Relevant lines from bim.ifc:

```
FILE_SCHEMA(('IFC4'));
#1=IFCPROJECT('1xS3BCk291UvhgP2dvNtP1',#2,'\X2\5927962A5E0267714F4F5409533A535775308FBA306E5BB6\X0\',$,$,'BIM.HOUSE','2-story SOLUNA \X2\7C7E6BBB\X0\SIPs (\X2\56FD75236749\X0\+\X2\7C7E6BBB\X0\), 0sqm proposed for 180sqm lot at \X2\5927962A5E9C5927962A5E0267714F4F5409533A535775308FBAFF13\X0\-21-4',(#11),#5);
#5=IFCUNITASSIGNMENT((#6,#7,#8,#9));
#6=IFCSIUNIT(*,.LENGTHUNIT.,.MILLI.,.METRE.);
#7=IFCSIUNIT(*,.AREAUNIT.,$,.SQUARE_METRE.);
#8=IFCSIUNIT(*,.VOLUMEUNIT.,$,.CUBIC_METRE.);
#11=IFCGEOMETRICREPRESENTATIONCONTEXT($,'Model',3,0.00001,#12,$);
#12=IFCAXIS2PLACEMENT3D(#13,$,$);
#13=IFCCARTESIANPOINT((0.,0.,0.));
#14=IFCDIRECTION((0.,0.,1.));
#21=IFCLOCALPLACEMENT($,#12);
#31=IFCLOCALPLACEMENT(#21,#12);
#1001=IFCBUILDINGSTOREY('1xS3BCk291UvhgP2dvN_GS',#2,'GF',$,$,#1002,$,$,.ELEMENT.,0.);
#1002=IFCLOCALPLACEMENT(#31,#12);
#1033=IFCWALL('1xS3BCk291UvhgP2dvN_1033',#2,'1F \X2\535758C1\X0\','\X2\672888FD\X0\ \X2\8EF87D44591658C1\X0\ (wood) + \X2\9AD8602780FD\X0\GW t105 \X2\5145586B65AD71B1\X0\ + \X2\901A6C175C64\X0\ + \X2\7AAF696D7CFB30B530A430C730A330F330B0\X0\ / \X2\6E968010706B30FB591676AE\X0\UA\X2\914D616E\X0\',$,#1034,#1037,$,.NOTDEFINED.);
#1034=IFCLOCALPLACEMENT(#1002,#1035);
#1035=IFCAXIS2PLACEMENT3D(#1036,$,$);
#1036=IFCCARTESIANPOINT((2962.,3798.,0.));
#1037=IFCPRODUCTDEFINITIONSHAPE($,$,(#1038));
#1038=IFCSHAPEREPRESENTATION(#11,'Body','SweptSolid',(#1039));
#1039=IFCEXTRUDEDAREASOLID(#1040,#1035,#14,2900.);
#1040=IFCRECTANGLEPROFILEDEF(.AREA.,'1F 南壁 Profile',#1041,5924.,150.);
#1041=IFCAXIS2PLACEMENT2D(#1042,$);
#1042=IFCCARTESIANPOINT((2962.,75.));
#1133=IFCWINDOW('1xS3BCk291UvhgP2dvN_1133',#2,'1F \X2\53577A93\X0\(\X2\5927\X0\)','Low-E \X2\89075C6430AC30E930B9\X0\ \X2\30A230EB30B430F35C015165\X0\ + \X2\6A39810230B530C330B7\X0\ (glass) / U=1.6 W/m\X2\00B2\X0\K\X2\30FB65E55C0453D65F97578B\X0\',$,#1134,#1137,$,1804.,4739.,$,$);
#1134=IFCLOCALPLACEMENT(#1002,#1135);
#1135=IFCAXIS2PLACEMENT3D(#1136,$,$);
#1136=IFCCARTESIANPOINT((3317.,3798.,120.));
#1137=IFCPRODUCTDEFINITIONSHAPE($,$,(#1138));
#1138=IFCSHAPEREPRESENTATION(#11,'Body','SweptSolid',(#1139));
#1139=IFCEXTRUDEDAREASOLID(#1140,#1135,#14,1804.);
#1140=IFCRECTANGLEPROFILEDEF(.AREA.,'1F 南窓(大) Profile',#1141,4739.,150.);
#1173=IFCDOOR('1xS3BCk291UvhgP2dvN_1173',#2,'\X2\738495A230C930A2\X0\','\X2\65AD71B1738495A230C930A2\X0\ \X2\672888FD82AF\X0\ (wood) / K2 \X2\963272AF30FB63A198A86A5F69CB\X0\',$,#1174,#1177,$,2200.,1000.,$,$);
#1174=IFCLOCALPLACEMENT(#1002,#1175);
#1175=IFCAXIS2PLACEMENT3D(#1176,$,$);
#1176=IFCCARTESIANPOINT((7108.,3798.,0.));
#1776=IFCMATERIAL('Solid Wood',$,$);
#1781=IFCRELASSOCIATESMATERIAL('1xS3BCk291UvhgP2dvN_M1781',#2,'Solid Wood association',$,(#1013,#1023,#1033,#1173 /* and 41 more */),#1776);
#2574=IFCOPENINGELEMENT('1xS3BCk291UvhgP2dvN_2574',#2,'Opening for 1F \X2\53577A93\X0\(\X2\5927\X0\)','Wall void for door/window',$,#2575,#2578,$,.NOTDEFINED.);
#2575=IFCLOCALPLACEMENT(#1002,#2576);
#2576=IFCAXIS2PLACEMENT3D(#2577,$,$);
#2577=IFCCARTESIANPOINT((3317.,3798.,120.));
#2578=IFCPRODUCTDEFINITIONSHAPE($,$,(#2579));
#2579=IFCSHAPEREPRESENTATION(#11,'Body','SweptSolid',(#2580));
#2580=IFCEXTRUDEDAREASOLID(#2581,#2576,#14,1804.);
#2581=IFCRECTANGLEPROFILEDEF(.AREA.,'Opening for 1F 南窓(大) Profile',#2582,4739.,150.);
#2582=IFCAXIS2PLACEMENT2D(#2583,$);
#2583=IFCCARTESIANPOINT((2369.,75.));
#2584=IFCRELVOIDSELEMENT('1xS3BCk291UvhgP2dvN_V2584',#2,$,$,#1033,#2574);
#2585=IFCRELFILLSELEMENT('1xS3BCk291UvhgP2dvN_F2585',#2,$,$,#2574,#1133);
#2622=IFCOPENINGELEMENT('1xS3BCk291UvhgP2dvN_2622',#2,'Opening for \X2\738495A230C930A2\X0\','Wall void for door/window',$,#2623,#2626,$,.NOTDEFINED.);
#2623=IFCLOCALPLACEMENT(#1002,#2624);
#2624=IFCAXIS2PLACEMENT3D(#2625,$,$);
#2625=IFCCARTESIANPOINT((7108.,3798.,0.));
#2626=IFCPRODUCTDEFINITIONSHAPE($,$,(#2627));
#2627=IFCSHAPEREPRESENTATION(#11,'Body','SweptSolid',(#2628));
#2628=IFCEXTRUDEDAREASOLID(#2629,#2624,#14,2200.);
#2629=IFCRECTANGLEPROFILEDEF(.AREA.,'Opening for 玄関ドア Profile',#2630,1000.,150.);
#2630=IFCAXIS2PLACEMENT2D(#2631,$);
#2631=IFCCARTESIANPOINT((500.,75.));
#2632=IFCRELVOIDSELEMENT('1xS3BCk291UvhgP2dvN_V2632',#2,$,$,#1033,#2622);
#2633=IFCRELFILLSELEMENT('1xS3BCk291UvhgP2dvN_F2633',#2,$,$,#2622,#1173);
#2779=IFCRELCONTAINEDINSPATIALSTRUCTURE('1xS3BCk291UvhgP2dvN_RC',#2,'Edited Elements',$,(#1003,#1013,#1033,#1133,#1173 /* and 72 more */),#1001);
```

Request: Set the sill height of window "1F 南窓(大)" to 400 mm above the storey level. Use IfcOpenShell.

```python
import numpy as np
import ifcopenshell
import ifcopenshell.api.geometry
import ifcopenshell.geom
import ifcopenshell.util.element
import ifcopenshell.util.placement
import ifcopenshell.util.shape
import ifcopenshell.util.unit

model = ifcopenshell.open("bim.ifc")
unit_scale = ifcopenshell.util.unit.calculate_unit_scale(model)

window = model.by_guid("1xS3BCk291UvhgP2dvN_1133")
opening = window.FillsVoids[0].RelatingOpeningElement
storey = ifcopenshell.util.element.get_container(window, ifc_class="IfcBuildingStorey")
level = ifcopenshell.util.placement.get_local_placement(storey.ObjectPlacement)[2, 3]

# The opening's origin need not be at the sill, so measure its lowest point.
shape = ifcopenshell.geom.create_shape(ifcopenshell.geom.settings(), opening)
bottom = ifcopenshell.util.shape.get_shape_bottom_elevation(shape, shape.geometry) / unit_scale
dz = level + 400.0 - bottom

shift = np.array([0.0, 0.0, dz])
# The window is not placed relative to its opening, so move both.
for product in (opening, window):
    matrix = ifcopenshell.util.placement.get_local_placement(product.ObjectPlacement)
    matrix[:3, 3] += shift
    ifcopenshell.api.geometry.edit_object_placement(model, product=product, matrix=matrix, is_si=False)

print(f"moved by {dz * unit_scale:+.3f} m")

model.write("bim_updated.ifc")
```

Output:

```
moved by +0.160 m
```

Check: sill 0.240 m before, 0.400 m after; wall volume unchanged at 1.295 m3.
